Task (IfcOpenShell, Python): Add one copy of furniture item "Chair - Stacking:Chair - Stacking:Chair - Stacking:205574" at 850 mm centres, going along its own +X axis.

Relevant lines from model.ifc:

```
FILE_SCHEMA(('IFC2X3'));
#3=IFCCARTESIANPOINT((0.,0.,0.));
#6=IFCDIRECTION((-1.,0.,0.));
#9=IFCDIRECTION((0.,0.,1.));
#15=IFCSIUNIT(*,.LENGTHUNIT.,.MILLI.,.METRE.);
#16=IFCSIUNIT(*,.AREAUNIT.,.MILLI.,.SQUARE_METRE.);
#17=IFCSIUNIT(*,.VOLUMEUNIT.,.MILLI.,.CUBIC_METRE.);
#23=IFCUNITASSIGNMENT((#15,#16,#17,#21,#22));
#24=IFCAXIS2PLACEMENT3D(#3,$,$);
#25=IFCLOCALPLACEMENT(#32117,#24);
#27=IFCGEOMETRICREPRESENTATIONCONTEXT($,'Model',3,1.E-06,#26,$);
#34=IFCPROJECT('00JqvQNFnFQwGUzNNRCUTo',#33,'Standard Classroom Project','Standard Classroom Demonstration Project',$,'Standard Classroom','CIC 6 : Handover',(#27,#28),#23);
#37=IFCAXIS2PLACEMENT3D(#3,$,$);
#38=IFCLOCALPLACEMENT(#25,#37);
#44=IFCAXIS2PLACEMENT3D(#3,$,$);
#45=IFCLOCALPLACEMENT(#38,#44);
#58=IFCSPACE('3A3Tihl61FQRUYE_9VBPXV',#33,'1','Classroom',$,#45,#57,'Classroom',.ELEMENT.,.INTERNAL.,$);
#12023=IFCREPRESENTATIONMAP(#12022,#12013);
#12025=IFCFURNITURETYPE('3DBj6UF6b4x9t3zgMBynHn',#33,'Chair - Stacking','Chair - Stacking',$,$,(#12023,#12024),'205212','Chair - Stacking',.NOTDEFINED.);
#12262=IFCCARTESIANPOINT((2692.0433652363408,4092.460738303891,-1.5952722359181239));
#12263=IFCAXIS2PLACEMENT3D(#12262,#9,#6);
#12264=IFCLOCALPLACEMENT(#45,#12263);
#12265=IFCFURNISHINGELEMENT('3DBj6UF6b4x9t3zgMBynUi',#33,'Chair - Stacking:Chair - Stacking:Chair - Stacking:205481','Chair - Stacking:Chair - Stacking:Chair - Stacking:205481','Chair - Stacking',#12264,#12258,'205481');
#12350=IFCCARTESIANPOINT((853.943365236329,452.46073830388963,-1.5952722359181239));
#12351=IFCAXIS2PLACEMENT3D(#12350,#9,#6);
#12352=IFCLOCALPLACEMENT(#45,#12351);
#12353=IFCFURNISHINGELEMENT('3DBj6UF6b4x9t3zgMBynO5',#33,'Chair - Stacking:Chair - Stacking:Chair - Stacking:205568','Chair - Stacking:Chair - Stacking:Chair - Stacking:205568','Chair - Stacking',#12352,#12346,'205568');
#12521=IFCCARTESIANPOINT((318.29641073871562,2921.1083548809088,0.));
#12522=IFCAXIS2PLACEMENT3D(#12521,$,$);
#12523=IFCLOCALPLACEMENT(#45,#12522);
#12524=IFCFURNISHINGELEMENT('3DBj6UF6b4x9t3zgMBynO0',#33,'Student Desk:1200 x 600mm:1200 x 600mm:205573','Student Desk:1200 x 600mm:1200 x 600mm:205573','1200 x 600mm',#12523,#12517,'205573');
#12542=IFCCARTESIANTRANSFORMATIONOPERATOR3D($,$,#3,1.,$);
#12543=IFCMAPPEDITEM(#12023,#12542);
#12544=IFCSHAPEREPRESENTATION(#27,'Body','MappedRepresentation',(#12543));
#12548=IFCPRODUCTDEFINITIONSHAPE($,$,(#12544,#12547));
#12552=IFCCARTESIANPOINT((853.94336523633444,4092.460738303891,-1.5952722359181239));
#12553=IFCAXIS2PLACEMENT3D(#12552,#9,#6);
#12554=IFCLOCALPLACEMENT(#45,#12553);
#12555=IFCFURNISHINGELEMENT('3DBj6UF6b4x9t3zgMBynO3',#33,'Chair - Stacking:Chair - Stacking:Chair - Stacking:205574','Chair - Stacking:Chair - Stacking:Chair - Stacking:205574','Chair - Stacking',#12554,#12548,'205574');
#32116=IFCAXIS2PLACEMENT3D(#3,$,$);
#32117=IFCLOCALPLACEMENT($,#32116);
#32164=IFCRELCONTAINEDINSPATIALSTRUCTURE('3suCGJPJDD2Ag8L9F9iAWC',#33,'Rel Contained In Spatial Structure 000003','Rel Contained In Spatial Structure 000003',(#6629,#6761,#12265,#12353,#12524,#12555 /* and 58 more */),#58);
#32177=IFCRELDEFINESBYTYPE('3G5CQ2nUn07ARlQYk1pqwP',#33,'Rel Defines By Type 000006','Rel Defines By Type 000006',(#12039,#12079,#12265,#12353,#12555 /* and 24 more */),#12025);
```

```python
import ifcopenshell
import ifcopenshell.api.geometry
import ifcopenshell.api.root
import ifcopenshell.util.element
import ifcopenshell.util.placement
import ifcopenshell.util.unit

model = ifcopenshell.open("model.ifc")
unit_scale = ifcopenshell.util.unit.calculate_unit_scale(model)


def reuse_history(source, copy):
    """copy_class also copies each property set's owner history, people and application; keep the originals."""
    for rel in copy.IsDefinedBy:
        if rel.is_a("IfcRelDefinesByProperties") and (history := rel.RelatingPropertyDefinition.OwnerHistory):
            rel.RelatingPropertyDefinition.OwnerHistory = source.OwnerHistory
            ifcopenshell.util.element.remove_deep2(model, history)


source = model.by_guid("3DBj6UF6b4x9t3zgMBynO3")
base = ifcopenshell.util.placement.get_local_placement(source.ObjectPlacement)
step = base[:3, 0] * 0.85 / unit_scale

for i in range(1, 2):
    copy = ifcopenshell.api.root.copy_class(model, product=source)
    copy.Representation = ifcopenshell.util.element.copy_deep(
        model, source.Representation, exclude=["IfcGeometricRepresentationContext", "IfcRepresentationMap"]
    )
    copy.Name = "Chair - Stacking:Chair - Stacking:Chair - Stacking"
    copy.Tag = None
    reuse_history(source, copy)
    matrix = base.copy()
    matrix[:3, 3] += i * step
    print("added at", matrix[:3, 3].round(3) + 0.0)
    ifcopenshell.api.geometry.edit_object_placement(model, product=copy, matrix=matrix, is_si=False)

model.write("model-out.ifc")
```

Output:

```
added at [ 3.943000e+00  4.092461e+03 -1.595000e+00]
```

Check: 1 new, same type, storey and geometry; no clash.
